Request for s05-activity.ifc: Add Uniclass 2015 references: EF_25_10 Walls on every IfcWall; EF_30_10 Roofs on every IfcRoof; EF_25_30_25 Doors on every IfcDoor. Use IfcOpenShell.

First a look at what the model holds.

```python
import ifcopenshell

model = ifcopenshell.open("s05-activity.ifc")
print(model.schema)
print("classifications:", [c.Name for c in model.by_type("IfcClassification")])
for ifc_class in ("IfcDoor", "IfcRoof", "IfcStair", "IfcWall", "IfcWindow"):
    print(ifc_class, len(model.by_type(ifc_class)))
```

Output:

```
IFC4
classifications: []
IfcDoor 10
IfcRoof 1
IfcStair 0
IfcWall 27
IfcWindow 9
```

```python
import ifcopenshell
import ifcopenshell.api.classification

model = ifcopenshell.open("s05-activity.ifc")

system = ifcopenshell.api.classification.add_classification(model, classification="Uniclass 2015")

codes = {
    "IfcWall": ("EF_25_10", "Walls"),
    "IfcRoof": ("EF_30_10", "Roofs"),
    "IfcDoor": ("EF_25_30_25", "Doors"),
}
for ifc_class, (code, name) in codes.items():
    products = model.by_type(ifc_class)
    ifcopenshell.api.classification.add_reference(
        model, products=products, classification=system, identification=code, name=name
    )
    print(code, len(products))

model.write("s05-activity_rev.ifc")
```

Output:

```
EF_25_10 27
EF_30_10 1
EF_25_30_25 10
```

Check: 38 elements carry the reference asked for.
